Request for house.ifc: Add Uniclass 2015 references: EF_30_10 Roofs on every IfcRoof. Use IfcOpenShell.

First a look at what the model holds.

```python
import ifcopenshell

model = ifcopenshell.open("house.ifc")
print(model.schema)
print("classifications:", [c.Name for c in model.by_type("IfcClassification")])
for ifc_class in ("IfcDoor", "IfcRoof", "IfcStair", "IfcWall", "IfcWindow"):
    print(ifc_class, len(model.by_type(ifc_class)))
```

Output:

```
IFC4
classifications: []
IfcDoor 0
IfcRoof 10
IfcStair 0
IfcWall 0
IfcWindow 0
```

```python
import ifcopenshell
import ifcopenshell.api.classification

model = ifcopenshell.open("house.ifc")

system = ifcopenshell.api.classification.add_classification(model, classification="Uniclass 2015")

codes = {
    "IfcRoof": ("EF_30_10", "Roofs"),
}
for ifc_class, (code, name) in codes.items():
    products = model.by_type(ifc_class)
    ifcopenshell.api.classification.add_reference(
        model, products=products, classification=system, identification=code, name=name
    )
    print(code, len(products))

model.write("house-out.ifc")
```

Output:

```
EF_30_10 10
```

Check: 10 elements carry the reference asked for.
